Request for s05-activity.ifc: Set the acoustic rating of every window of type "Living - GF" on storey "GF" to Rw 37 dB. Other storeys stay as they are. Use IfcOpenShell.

First a look at what the model holds.

```python
import ifcopenshell
import ifcopenshell.util.element

model = ifcopenshell.open("s05-activity.ifc")
print(model.schema)
storey = next(s for s in model.by_type("IfcBuildingStorey") if s.Name == "GF")
windows = [e for e in ifcopenshell.util.element.get_decomposition(storey) if e.is_a("IfcWindow")]
seen = {}
for e in windows:
    element_type = ifcopenshell.util.element.get_type(e)
    key = (element_type.Name if element_type != e and element_type else None, ifcopenshell.util.element.get_pset(e, "Pset_WindowCommon", "AcousticRating"))
    seen[key] = seen.get(key, 0) + 1
for (name, value), count in sorted(seen.items(), key=str):
    print(count, "x", name, "|", value)
```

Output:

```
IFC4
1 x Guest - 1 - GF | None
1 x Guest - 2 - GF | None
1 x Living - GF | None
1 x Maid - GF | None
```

```python
import ifcopenshell
import ifcopenshell.api.pset
import ifcopenshell.util.element

model = ifcopenshell.open("s05-activity.ifc")

storey = next(s for s in model.by_type("IfcBuildingStorey") if s.Name == "GF")
windows = [e for e in ifcopenshell.util.element.get_decomposition(storey) if e.is_a("IfcWindow")]

count = 0
for e in windows:
    element_type = ifcopenshell.util.element.get_type(e)
    if element_type in (None, e) or element_type.Name != "Living - GF":
        continue
    # add_pset returns the element's existing set when there is one.
    pset = ifcopenshell.api.pset.add_pset(model, product=e, name="Pset_WindowCommon")
    ifcopenshell.api.pset.edit_pset(model, pset=pset, properties={"AcousticRating": "Rw 37 dB"})
    count += 1

print(count, "windows updated")

model.write("s05-activity_rev.ifc")
```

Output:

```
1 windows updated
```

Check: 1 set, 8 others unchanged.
